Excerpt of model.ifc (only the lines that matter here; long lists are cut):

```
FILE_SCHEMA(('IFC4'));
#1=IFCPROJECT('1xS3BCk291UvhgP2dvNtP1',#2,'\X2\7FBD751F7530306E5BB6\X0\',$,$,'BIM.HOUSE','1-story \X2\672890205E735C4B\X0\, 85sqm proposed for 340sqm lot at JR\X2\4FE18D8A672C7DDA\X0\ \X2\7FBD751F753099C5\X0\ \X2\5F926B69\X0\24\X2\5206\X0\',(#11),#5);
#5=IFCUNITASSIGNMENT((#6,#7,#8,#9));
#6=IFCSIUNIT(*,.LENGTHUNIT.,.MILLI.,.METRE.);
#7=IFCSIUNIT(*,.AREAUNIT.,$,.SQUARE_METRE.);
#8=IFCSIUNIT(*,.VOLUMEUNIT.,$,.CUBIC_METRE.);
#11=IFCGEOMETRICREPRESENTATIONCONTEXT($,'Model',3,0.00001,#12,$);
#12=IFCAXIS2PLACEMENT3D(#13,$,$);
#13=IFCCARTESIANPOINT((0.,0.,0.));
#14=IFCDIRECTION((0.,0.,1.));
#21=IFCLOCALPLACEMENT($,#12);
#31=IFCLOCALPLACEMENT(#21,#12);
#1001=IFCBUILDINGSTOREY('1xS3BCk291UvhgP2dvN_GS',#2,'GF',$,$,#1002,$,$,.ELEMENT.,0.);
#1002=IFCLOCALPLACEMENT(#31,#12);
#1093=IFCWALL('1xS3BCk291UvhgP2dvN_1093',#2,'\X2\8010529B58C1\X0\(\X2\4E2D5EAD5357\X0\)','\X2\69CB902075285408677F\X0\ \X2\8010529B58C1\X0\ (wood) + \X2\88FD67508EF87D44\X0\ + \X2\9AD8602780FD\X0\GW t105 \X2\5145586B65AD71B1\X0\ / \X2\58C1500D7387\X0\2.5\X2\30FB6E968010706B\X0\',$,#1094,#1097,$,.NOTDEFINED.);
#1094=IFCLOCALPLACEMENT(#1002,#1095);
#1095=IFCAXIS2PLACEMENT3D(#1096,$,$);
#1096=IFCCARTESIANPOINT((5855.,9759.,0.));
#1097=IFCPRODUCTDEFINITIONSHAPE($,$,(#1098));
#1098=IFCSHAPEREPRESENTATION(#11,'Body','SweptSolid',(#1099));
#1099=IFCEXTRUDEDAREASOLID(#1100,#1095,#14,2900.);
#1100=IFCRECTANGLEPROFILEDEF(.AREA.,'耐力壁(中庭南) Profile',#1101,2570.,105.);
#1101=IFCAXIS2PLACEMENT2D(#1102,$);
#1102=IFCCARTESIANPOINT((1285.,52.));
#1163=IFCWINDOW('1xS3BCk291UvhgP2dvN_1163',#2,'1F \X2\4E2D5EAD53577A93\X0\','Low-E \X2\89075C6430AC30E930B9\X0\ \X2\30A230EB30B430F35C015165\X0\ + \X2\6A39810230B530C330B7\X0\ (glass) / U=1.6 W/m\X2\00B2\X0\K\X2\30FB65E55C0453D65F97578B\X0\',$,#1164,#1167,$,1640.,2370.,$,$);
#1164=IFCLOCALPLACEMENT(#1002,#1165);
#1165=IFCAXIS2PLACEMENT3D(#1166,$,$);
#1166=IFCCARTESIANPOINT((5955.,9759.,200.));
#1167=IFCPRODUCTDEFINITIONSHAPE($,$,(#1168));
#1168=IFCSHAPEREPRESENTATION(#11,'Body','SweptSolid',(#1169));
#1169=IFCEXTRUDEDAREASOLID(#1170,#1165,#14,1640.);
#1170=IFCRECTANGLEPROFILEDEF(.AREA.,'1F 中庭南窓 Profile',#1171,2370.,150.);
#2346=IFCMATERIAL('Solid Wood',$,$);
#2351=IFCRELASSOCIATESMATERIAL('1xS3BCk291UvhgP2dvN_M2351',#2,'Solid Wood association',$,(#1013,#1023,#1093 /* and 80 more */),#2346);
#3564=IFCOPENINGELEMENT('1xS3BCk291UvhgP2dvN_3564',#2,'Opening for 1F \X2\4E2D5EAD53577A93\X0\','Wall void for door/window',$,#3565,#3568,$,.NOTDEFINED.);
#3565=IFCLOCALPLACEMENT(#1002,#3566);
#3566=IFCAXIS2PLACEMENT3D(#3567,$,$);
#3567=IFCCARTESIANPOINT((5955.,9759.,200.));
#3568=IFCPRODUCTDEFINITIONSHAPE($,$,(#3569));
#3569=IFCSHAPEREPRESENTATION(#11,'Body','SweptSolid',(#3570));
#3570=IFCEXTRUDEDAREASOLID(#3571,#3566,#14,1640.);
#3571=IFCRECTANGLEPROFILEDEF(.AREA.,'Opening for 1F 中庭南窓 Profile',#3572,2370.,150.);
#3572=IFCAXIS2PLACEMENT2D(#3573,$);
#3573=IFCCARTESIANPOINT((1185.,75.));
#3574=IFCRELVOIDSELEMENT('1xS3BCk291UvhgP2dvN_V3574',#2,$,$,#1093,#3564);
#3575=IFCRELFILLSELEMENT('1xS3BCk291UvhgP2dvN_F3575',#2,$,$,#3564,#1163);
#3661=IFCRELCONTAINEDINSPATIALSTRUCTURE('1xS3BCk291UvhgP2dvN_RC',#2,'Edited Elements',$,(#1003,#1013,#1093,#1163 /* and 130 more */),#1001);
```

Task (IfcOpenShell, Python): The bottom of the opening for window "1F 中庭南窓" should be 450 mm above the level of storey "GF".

```python
import numpy as np
import ifcopenshell
import ifcopenshell.api.geometry
import ifcopenshell.geom
import ifcopenshell.util.element
import ifcopenshell.util.placement
import ifcopenshell.util.shape
import ifcopenshell.util.unit

model = ifcopenshell.open("model.ifc")
unit_scale = ifcopenshell.util.unit.calculate_unit_scale(model)

window = model.by_guid("1xS3BCk291UvhgP2dvN_1163")
opening = window.FillsVoids[0].RelatingOpeningElement
storey = ifcopenshell.util.element.get_container(window, ifc_class="IfcBuildingStorey")
level = ifcopenshell.util.placement.get_local_placement(storey.ObjectPlacement)[2, 3]

# The opening's origin need not be at the sill, so measure its lowest point.
shape = ifcopenshell.geom.create_shape(ifcopenshell.geom.settings(), opening)
bottom = ifcopenshell.util.shape.get_shape_bottom_elevation(shape, shape.geometry) / unit_scale
dz = level + 0.45 / unit_scale - bottom

shift = np.array([0.0, 0.0, dz])
# The window is not placed relative to its opening, so move both.
for product in (opening, window):
    matrix = ifcopenshell.util.placement.get_local_placement(product.ObjectPlacement)
    matrix[:3, 3] += shift
    ifcopenshell.api.geometry.edit_object_placement(model, product=product, matrix=matrix, is_si=False)

print(f"moved by {dz * unit_scale:+.3f} m")

model.write("model_edited.ifc")
```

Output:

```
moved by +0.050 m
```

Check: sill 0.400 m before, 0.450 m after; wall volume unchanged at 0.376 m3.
